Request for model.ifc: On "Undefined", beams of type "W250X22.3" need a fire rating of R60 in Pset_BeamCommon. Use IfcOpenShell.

First a look at what the model holds.

```python
import ifcopenshell
import ifcopenshell.util.element

model = ifcopenshell.open("model.ifc")
print(model.schema)
storey = next(s for s in model.by_type("IfcBuildingStorey") if s.Name == "Undefined")
beams = [e for e in ifcopenshell.util.element.get_decomposition(storey) if e.is_a("IfcBeam")]
seen = {}
for e in beams:
    element_type = ifcopenshell.util.element.get_type(e)
    key = (element_type.Name if element_type != e and element_type else None, ifcopenshell.util.element.get_pset(e, "Pset_BeamCommon", "FireRating"))
    seen[key] = seen.get(key, 0) + 1
for (name, value), count in sorted(seen.items(), key=str):
    print(count, "x", name, "|", value)
```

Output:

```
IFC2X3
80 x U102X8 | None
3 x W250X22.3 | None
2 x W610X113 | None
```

```python
import ifcopenshell
import ifcopenshell.api.pset
import ifcopenshell.util.element

model = ifcopenshell.open("model.ifc")

storey = next(s for s in model.by_type("IfcBuildingStorey") if s.Name == "Undefined")
beams = [e for e in ifcopenshell.util.element.get_decomposition(storey) if e.is_a("IfcBeam")]

count = 0
for e in beams:
    element_type = ifcopenshell.util.element.get_type(e)
    if element_type in (None, e) or element_type.Name != "W250X22.3":
        continue
    found = ifcopenshell.util.element.get_pset(e, "Pset_BeamCommon", should_inherit=False)
    if found:
        pset = model.by_id(found["id"])
        if len(ifcopenshell.util.element.get_elements_by_pset(pset)) > 1:
            pset = ifcopenshell.api.pset.unshare_pset(model, products=[e], pset=pset)[0]
    else:
        pset = ifcopenshell.api.pset.add_pset(model, product=e, name="Pset_BeamCommon")
    ifcopenshell.api.pset.edit_pset(model, pset=pset, properties={"FireRating": "R60"})
    count += 1

print(count, "beams updated")

model.write("model_edited.ifc")
```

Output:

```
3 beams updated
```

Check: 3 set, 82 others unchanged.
